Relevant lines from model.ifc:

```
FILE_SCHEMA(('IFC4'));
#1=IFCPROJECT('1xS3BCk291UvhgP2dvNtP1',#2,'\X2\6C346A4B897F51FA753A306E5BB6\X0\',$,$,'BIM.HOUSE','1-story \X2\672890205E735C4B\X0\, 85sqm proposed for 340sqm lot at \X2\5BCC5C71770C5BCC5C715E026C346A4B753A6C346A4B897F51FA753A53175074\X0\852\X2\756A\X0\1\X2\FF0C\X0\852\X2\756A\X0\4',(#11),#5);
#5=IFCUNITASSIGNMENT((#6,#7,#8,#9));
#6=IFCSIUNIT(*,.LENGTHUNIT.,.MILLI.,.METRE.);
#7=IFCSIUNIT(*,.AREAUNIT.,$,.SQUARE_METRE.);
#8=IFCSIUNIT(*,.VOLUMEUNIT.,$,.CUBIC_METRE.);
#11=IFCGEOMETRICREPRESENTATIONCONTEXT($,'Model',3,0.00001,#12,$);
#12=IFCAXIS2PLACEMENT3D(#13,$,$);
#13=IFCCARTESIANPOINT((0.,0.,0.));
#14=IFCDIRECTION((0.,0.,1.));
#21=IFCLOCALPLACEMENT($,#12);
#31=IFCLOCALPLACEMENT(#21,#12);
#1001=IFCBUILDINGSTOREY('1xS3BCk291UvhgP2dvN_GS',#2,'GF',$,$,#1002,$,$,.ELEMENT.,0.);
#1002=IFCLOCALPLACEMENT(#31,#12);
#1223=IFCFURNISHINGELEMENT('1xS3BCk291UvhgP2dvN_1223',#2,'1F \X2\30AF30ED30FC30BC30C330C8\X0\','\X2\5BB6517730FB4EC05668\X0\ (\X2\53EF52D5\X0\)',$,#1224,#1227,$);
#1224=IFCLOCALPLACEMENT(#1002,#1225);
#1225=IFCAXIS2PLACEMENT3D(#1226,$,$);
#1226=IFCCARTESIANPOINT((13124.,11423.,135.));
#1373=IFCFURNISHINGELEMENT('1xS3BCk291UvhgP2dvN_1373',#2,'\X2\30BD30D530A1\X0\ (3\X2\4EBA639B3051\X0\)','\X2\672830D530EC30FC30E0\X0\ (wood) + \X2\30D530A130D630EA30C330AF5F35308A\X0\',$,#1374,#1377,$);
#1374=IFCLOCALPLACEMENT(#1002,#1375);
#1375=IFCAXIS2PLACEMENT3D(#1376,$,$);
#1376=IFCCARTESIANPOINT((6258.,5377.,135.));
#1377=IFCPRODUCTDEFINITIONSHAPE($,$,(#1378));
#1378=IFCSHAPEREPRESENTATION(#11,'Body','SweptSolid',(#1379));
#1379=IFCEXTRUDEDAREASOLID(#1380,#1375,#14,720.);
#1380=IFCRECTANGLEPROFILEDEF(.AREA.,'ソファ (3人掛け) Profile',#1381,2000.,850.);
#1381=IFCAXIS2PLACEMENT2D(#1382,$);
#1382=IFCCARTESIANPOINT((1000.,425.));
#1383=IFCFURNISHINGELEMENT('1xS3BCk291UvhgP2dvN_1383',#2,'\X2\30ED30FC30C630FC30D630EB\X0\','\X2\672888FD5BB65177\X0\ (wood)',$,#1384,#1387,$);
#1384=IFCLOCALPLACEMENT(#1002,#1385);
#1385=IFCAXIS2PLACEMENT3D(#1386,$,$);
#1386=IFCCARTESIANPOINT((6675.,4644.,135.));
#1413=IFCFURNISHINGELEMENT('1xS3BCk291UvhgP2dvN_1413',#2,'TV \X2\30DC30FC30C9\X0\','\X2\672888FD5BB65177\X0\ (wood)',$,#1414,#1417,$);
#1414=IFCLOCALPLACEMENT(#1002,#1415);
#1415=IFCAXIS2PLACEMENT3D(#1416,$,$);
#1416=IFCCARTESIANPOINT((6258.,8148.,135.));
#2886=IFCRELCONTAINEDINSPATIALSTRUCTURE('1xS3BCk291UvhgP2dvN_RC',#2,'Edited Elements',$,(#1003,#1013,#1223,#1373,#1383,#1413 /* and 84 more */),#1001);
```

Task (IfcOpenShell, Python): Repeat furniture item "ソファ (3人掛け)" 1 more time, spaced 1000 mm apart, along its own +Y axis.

```python
import ifcopenshell
import ifcopenshell.api.geometry
import ifcopenshell.api.root
import ifcopenshell.util.element
import ifcopenshell.util.placement

model = ifcopenshell.open("model.ifc")


def reuse_history(source, copy):
    """copy_class also copies each property set's owner history, people and application; keep the originals."""
    for rel in copy.IsDefinedBy:
        if rel.is_a("IfcRelDefinesByProperties") and (history := rel.RelatingPropertyDefinition.OwnerHistory):
            rel.RelatingPropertyDefinition.OwnerHistory = source.OwnerHistory
            ifcopenshell.util.element.remove_deep2(model, history)


source = model.by_guid("1xS3BCk291UvhgP2dvN_1373")
base = ifcopenshell.util.placement.get_local_placement(source.ObjectPlacement)
step = base[:3, 1] * 1000.0

for i in range(1, 2):
    copy = ifcopenshell.api.root.copy_class(model, product=source)
    copy.Representation = ifcopenshell.util.element.copy_deep(
        model, source.Representation, exclude=["IfcGeometricRepresentationContext", "IfcRepresentationMap"]
    )
    reuse_history(source, copy)
    matrix = base.copy()
    matrix[:3, 3] += i * step
    print("added at", matrix[:3, 3].round(3) + 0.0)
    ifcopenshell.api.geometry.edit_object_placement(model, product=copy, matrix=matrix, is_si=False)

model.write("model_updated.ifc")
```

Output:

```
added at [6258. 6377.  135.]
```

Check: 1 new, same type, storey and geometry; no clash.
